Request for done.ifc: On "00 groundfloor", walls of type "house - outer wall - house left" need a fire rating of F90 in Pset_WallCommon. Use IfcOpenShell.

First a look at what the model holds.

```python
import ifcopenshell
import ifcopenshell.util.element

model = ifcopenshell.open("done.ifc")
print(model.schema)
storey = next(s for s in model.by_type("IfcBuildingStorey") if s.Name == "00 groundfloor")
walls = [e for e in ifcopenshell.util.element.get_decomposition(storey) if e.is_a("IfcWall")]
seen = {}
for e in walls:
    element_type = ifcopenshell.util.element.get_type(e)
    key = (element_type.Name if element_type != e and element_type else None, ifcopenshell.util.element.get_pset(e, "Pset_WallCommon", "FireRating"))
    seen[key] = seen.get(key, 0) + 1
for (name, value), count in sorted(seen.items(), key=str):
    print(count, "x", name, "|", value)
```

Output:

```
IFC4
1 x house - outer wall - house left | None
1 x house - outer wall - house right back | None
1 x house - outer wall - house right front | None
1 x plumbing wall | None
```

```python
import ifcopenshell
import ifcopenshell.api.pset
import ifcopenshell.util.element

model = ifcopenshell.open("done.ifc")

storey = next(s for s in model.by_type("IfcBuildingStorey") if s.Name == "00 groundfloor")
walls = [e for e in ifcopenshell.util.element.get_decomposition(storey) if e.is_a("IfcWall")]

count = 0
for e in walls:
    element_type = ifcopenshell.util.element.get_type(e)
    if element_type in (None, e) or element_type.Name != "house - outer wall - house left":
        continue
    # add_pset returns the element's existing set when there is one.
    pset = ifcopenshell.api.pset.add_pset(model, product=e, name="Pset_WallCommon")
    ifcopenshell.api.pset.edit_pset(model, pset=pset, properties={"FireRating": "F90"})
    count += 1

print(count, "walls updated")

model.write("done_v2.ifc")
```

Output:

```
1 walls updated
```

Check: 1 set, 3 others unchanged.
